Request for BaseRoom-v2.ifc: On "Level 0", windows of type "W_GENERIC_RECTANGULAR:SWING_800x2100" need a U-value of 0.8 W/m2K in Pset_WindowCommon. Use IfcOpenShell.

First a look at what the model holds.

```python
import ifcopenshell
import ifcopenshell.util.element

model = ifcopenshell.open("BaseRoom-v2.ifc")
print(model.schema)
storey = next(s for s in model.by_type("IfcBuildingStorey") if s.Name == "Level 0")
windows = [e for e in ifcopenshell.util.element.get_decomposition(storey) if e.is_a("IfcWindow")]
seen = {}
for e in windows:
    element_type = ifcopenshell.util.element.get_type(e)
    key = (element_type.Name if element_type != e and element_type else None, ifcopenshell.util.element.get_pset(e, "Pset_WindowCommon", "ThermalTransmittance"))
    seen[key] = seen.get(key, 0) + 1
for (name, value), count in sorted(seen.items(), key=str):
    print(count, "x", name, "|", value)
```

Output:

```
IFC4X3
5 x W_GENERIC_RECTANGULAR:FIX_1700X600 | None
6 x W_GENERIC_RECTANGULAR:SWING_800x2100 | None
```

```python
import ifcopenshell
import ifcopenshell.api.pset
import ifcopenshell.util.element

model = ifcopenshell.open("BaseRoom-v2.ifc")

storey = next(s for s in model.by_type("IfcBuildingStorey") if s.Name == "Level 0")
windows = [e for e in ifcopenshell.util.element.get_decomposition(storey) if e.is_a("IfcWindow")]

count = 0
for e in windows:
    element_type = ifcopenshell.util.element.get_type(e)
    if element_type in (None, e) or element_type.Name != "W_GENERIC_RECTANGULAR:SWING_800x2100":
        continue
    # add_pset returns the element's existing set when there is one.
    pset = ifcopenshell.api.pset.add_pset(model, product=e, name="Pset_WindowCommon")
    ifcopenshell.api.pset.edit_pset(model, pset=pset, properties={"ThermalTransmittance": 0.8})
    count += 1

print(count, "windows updated")

model.write("BaseRoom-v2-out.ifc")
```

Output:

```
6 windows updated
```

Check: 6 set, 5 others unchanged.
